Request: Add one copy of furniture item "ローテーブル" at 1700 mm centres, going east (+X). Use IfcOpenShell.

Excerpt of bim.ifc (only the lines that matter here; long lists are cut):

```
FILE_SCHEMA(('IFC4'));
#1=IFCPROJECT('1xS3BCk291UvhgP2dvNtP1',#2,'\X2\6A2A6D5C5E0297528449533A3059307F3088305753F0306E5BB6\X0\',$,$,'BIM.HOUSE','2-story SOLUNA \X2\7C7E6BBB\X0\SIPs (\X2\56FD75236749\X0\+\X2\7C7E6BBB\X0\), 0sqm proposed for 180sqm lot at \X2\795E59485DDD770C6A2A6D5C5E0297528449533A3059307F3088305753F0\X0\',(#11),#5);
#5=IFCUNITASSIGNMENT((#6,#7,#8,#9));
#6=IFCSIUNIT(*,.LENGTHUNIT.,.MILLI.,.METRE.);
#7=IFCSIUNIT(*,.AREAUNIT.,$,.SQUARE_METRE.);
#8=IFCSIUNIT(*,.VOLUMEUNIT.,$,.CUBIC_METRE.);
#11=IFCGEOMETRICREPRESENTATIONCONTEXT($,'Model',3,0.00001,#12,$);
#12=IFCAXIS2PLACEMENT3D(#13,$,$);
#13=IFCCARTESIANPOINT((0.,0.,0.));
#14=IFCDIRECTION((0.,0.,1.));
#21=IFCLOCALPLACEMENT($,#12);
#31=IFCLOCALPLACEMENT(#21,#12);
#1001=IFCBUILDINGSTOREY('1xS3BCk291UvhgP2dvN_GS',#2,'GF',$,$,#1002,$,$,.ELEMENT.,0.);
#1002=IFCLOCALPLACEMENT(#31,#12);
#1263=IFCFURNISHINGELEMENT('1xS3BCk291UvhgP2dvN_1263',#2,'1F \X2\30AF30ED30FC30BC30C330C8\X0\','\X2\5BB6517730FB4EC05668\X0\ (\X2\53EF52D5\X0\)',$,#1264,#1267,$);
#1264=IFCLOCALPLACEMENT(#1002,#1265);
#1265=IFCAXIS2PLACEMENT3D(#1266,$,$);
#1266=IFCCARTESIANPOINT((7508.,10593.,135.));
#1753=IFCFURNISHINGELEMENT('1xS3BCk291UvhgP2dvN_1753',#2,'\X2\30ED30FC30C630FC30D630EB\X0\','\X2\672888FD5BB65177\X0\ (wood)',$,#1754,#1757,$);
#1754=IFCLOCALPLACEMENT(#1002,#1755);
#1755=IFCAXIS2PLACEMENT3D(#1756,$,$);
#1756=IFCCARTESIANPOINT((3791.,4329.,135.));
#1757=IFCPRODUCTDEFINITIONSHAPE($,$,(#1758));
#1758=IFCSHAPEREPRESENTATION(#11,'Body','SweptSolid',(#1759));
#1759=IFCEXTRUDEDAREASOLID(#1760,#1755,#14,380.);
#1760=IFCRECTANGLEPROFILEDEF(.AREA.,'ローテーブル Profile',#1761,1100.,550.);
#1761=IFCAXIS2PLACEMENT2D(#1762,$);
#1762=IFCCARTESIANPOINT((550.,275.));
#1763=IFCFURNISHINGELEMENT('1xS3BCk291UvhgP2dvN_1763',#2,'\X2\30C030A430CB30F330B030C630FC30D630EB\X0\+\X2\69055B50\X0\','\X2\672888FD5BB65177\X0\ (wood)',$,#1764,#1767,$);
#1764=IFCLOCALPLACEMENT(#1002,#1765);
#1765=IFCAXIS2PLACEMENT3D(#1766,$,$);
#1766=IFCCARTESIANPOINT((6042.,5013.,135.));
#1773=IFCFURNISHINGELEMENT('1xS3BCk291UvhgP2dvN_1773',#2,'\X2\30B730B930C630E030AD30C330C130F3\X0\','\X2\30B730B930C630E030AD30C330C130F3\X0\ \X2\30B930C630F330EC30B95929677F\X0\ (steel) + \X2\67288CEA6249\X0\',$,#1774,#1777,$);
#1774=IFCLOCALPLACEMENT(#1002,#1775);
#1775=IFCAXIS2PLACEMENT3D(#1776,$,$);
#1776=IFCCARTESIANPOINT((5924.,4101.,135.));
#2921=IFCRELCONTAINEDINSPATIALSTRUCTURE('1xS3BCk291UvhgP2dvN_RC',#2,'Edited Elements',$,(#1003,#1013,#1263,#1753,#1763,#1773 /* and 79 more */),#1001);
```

```python
import numpy as np
import ifcopenshell
import ifcopenshell.api.geometry
import ifcopenshell.api.root
import ifcopenshell.util.element
import ifcopenshell.util.placement
import ifcopenshell.util.unit

model = ifcopenshell.open("bim.ifc")
unit_scale = ifcopenshell.util.unit.calculate_unit_scale(model)


def reuse_history(source, copy):
    """copy_class also copies each property set's owner history, people and application; keep the originals."""
    for rel in copy.IsDefinedBy:
        if rel.is_a("IfcRelDefinesByProperties") and (history := rel.RelatingPropertyDefinition.OwnerHistory):
            rel.RelatingPropertyDefinition.OwnerHistory = source.OwnerHistory
            ifcopenshell.util.element.remove_deep2(model, history)


source = model.by_id(1753)
base = ifcopenshell.util.placement.get_local_placement(source.ObjectPlacement)
step = np.array([1.0, 0.0, 0.0]) * 1.7 / unit_scale

for i in range(1, 2):
    copy = ifcopenshell.api.root.copy_class(model, product=source)
    copy.Representation = ifcopenshell.util.element.copy_deep(
        model, source.Representation, exclude=["IfcGeometricRepresentationContext", "IfcRepresentationMap"]
    )
    reuse_history(source, copy)
    matrix = base.copy()
    matrix[:3, 3] += i * step
    print("added at", matrix[:3, 3].round(3) + 0.0)
    ifcopenshell.api.geometry.edit_object_placement(model, product=copy, matrix=matrix, is_si=False)

model.write("bim_v2.ifc")
```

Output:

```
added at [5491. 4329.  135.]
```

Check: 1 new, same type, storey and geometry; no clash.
